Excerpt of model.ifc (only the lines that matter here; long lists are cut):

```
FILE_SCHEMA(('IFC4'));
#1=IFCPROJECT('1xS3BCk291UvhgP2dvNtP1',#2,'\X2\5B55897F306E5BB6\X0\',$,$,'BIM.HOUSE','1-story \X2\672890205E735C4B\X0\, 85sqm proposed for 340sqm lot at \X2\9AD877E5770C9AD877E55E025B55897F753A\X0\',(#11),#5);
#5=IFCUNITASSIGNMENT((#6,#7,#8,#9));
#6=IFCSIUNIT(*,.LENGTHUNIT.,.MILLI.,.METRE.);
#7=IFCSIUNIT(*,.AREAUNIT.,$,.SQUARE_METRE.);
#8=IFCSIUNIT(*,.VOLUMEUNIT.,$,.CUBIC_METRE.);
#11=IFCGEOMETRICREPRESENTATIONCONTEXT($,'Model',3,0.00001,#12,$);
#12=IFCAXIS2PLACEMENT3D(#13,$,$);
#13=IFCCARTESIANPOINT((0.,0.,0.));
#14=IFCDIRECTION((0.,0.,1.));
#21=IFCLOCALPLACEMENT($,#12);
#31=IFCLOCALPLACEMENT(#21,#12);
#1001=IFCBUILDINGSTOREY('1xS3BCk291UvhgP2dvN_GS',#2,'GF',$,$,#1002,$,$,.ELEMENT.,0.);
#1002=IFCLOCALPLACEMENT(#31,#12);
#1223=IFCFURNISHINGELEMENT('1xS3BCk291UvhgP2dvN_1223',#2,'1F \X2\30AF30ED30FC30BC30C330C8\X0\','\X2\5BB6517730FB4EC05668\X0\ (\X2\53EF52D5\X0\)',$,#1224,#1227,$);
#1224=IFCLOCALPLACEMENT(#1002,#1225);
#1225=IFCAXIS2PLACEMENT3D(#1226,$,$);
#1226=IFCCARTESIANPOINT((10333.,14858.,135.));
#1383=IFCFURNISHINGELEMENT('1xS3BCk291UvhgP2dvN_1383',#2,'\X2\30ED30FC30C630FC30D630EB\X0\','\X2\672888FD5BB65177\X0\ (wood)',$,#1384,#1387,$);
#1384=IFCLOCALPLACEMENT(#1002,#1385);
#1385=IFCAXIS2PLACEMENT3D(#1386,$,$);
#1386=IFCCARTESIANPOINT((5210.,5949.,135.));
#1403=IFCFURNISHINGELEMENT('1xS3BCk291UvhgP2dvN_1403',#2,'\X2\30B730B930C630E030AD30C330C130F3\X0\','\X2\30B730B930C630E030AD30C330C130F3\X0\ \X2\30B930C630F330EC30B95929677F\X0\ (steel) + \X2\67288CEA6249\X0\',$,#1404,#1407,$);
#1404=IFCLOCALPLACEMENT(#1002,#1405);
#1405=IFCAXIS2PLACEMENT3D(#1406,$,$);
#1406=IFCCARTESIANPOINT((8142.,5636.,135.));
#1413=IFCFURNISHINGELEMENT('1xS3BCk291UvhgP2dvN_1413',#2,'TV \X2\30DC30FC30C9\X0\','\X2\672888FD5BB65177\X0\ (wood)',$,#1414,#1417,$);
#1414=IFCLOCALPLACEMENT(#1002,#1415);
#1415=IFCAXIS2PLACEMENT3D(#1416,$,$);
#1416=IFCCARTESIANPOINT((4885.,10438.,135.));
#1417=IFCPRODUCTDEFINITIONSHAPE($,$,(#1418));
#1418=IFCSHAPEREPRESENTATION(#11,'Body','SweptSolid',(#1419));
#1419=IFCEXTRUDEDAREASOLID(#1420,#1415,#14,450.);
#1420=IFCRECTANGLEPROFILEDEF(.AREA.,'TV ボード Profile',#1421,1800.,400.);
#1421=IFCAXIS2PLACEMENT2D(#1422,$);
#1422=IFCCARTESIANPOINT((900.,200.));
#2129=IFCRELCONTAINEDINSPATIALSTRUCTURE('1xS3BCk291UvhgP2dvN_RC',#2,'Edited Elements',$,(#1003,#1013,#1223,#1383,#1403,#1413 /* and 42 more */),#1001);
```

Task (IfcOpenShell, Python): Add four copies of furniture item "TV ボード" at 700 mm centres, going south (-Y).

```python
import numpy as np
import ifcopenshell
import ifcopenshell.api.geometry
import ifcopenshell.api.root
import ifcopenshell.util.element
import ifcopenshell.util.placement

model = ifcopenshell.open("model.ifc")


def reuse_history(source, copy):
    """copy_class also copies each property set's owner history, people and application; keep the originals."""
    for rel in copy.IsDefinedBy:
        if rel.is_a("IfcRelDefinesByProperties") and (history := rel.RelatingPropertyDefinition.OwnerHistory):
            rel.RelatingPropertyDefinition.OwnerHistory = source.OwnerHistory
            ifcopenshell.util.element.remove_deep2(model, history)


source = model.by_id(1413)
base = ifcopenshell.util.placement.get_local_placement(source.ObjectPlacement)
step = np.array([0.0, -1.0, 0.0]) * 700.0

for i in range(1, 5):
    copy = ifcopenshell.api.root.copy_class(model, product=source)
    copy.Representation = ifcopenshell.util.element.copy_deep(
        model, source.Representation, exclude=["IfcGeometricRepresentationContext", "IfcRepresentationMap"]
    )
    reuse_history(source, copy)
    matrix = base.copy()
    matrix[:3, 3] += i * step
    print("added at", matrix[:3, 3].round(3) + 0.0)
    ifcopenshell.api.geometry.edit_object_placement(model, product=copy, matrix=matrix, is_si=False)

model.write("model_rev.ifc")
```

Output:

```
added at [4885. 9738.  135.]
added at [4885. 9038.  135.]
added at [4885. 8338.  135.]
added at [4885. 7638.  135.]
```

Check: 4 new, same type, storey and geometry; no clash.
